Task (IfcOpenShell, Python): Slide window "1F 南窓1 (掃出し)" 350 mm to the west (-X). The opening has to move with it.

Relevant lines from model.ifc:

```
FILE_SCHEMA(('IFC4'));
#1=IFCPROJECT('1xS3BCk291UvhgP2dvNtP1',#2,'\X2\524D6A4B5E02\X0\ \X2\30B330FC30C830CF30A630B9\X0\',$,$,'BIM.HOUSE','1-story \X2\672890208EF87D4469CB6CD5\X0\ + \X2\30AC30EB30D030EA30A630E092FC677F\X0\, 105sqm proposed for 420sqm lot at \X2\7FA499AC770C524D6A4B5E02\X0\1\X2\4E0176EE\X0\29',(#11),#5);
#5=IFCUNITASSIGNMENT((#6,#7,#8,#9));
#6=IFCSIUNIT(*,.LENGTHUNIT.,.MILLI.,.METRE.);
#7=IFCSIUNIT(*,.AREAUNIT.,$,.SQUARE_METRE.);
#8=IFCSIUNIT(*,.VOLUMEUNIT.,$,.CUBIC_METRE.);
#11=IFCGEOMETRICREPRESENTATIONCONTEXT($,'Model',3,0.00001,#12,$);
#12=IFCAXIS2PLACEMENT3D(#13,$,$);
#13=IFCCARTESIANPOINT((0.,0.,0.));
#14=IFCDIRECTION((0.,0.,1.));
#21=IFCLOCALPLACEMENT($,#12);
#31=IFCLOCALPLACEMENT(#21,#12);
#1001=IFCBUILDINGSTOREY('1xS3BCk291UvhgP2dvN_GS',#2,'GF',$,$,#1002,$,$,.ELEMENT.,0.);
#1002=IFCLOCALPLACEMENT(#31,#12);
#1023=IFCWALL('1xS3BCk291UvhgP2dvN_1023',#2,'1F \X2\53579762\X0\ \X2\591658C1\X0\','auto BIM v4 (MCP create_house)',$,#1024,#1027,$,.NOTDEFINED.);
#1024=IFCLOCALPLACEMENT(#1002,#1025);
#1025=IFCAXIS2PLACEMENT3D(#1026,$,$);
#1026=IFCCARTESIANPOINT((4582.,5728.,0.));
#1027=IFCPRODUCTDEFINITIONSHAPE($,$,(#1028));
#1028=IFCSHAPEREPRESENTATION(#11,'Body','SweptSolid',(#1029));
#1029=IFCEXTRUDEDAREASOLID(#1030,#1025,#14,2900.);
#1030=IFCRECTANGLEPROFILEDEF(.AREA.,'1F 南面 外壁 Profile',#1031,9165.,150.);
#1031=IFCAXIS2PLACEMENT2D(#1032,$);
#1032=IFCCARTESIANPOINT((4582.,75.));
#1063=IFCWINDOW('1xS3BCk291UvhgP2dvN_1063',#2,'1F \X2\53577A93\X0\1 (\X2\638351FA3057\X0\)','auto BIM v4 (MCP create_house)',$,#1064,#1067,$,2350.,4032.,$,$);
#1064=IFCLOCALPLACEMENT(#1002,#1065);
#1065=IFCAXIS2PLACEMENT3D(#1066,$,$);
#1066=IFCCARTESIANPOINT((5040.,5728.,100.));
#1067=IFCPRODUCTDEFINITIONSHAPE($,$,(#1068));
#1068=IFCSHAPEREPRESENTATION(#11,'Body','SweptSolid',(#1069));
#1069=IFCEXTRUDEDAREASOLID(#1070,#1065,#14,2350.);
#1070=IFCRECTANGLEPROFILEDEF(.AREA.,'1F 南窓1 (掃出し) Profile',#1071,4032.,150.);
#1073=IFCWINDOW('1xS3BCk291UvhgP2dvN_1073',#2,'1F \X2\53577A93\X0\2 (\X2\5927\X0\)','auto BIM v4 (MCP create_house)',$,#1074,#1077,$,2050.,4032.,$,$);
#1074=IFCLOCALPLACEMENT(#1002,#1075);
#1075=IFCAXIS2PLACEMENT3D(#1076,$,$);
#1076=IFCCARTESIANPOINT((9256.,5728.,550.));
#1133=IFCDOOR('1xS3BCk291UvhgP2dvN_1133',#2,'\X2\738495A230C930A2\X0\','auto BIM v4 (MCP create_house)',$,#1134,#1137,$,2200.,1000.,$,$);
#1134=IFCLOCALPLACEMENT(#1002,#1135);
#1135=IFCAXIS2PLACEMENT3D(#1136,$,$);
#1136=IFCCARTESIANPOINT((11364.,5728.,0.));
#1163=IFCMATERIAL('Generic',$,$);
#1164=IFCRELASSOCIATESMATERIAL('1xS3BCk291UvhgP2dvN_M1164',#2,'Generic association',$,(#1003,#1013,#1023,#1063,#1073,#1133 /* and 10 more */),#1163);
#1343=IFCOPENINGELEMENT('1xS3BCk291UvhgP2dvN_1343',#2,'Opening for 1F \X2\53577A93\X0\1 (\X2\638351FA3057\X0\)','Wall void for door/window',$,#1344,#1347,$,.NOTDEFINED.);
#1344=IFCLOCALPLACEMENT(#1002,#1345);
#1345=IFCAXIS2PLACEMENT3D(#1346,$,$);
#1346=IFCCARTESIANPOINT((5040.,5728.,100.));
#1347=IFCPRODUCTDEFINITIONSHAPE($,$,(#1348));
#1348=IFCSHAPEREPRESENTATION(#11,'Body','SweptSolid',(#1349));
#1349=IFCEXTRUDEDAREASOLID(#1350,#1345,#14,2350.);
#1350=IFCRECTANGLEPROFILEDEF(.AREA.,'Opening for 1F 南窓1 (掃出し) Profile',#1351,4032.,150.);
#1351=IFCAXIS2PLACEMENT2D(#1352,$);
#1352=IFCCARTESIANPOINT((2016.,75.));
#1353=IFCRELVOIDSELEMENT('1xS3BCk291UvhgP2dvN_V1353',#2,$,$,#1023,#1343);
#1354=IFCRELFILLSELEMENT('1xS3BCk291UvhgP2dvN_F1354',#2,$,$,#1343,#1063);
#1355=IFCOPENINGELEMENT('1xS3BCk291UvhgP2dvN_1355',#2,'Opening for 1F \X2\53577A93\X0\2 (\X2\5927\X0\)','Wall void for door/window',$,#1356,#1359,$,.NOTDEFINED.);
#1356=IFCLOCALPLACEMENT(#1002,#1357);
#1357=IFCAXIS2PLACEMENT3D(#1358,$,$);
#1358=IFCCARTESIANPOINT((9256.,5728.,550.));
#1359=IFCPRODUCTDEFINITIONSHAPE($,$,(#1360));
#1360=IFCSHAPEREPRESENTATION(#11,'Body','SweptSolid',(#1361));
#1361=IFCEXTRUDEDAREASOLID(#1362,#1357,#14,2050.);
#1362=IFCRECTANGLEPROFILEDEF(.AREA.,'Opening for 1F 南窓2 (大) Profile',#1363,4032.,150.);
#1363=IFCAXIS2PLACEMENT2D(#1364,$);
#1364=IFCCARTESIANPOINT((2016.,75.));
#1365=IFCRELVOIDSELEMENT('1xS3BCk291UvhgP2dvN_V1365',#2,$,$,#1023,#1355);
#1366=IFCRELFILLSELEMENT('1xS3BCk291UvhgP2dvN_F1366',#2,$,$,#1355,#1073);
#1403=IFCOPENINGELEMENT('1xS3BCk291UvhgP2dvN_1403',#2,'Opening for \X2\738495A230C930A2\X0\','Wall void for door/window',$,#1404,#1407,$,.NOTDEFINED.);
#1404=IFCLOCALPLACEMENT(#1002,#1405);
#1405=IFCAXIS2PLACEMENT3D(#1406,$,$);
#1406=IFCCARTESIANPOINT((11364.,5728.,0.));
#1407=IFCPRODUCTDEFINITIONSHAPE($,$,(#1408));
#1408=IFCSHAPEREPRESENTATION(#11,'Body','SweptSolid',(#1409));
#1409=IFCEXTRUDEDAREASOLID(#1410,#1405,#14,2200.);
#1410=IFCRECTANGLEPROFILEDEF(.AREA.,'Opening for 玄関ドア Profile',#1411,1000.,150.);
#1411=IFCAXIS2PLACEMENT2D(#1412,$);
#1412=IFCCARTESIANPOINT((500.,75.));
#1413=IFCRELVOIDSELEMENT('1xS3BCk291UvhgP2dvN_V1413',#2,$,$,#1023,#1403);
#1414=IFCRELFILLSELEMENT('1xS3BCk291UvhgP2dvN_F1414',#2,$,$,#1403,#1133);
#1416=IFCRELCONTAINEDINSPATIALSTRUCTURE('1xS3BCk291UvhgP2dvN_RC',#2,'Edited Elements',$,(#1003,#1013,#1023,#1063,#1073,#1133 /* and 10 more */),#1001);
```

```python
import ifcopenshell
import ifcopenshell.api.geometry
import ifcopenshell.util.placement

model = ifcopenshell.open("model.ifc")

window = model.by_id(1063)
opening = window.FillsVoids[0].RelatingOpeningElement
wall = opening.VoidsElements[0].RelatingBuildingElement

wall_matrix = ifcopenshell.util.placement.get_local_placement(wall.ObjectPlacement)
shift = wall_matrix[:3, 0] * -350.0
before = ifcopenshell.util.placement.get_local_placement(window.ObjectPlacement)[:3, 3].copy()

# The window is not placed relative to its opening, so move both.
for product in (opening, window):
    matrix = ifcopenshell.util.placement.get_local_placement(product.ObjectPlacement)
    matrix[:3, 3] += shift
    ifcopenshell.api.geometry.edit_object_placement(model, product=product, matrix=matrix, is_si=False)

after = ifcopenshell.util.placement.get_local_placement(window.ObjectPlacement)[:3, 3]
print("window moved by", (after - before).round(3) + 0.0)

model.write("model_updated.ifc")
```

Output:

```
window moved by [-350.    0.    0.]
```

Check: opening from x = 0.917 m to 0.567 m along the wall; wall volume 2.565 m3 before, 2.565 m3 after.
